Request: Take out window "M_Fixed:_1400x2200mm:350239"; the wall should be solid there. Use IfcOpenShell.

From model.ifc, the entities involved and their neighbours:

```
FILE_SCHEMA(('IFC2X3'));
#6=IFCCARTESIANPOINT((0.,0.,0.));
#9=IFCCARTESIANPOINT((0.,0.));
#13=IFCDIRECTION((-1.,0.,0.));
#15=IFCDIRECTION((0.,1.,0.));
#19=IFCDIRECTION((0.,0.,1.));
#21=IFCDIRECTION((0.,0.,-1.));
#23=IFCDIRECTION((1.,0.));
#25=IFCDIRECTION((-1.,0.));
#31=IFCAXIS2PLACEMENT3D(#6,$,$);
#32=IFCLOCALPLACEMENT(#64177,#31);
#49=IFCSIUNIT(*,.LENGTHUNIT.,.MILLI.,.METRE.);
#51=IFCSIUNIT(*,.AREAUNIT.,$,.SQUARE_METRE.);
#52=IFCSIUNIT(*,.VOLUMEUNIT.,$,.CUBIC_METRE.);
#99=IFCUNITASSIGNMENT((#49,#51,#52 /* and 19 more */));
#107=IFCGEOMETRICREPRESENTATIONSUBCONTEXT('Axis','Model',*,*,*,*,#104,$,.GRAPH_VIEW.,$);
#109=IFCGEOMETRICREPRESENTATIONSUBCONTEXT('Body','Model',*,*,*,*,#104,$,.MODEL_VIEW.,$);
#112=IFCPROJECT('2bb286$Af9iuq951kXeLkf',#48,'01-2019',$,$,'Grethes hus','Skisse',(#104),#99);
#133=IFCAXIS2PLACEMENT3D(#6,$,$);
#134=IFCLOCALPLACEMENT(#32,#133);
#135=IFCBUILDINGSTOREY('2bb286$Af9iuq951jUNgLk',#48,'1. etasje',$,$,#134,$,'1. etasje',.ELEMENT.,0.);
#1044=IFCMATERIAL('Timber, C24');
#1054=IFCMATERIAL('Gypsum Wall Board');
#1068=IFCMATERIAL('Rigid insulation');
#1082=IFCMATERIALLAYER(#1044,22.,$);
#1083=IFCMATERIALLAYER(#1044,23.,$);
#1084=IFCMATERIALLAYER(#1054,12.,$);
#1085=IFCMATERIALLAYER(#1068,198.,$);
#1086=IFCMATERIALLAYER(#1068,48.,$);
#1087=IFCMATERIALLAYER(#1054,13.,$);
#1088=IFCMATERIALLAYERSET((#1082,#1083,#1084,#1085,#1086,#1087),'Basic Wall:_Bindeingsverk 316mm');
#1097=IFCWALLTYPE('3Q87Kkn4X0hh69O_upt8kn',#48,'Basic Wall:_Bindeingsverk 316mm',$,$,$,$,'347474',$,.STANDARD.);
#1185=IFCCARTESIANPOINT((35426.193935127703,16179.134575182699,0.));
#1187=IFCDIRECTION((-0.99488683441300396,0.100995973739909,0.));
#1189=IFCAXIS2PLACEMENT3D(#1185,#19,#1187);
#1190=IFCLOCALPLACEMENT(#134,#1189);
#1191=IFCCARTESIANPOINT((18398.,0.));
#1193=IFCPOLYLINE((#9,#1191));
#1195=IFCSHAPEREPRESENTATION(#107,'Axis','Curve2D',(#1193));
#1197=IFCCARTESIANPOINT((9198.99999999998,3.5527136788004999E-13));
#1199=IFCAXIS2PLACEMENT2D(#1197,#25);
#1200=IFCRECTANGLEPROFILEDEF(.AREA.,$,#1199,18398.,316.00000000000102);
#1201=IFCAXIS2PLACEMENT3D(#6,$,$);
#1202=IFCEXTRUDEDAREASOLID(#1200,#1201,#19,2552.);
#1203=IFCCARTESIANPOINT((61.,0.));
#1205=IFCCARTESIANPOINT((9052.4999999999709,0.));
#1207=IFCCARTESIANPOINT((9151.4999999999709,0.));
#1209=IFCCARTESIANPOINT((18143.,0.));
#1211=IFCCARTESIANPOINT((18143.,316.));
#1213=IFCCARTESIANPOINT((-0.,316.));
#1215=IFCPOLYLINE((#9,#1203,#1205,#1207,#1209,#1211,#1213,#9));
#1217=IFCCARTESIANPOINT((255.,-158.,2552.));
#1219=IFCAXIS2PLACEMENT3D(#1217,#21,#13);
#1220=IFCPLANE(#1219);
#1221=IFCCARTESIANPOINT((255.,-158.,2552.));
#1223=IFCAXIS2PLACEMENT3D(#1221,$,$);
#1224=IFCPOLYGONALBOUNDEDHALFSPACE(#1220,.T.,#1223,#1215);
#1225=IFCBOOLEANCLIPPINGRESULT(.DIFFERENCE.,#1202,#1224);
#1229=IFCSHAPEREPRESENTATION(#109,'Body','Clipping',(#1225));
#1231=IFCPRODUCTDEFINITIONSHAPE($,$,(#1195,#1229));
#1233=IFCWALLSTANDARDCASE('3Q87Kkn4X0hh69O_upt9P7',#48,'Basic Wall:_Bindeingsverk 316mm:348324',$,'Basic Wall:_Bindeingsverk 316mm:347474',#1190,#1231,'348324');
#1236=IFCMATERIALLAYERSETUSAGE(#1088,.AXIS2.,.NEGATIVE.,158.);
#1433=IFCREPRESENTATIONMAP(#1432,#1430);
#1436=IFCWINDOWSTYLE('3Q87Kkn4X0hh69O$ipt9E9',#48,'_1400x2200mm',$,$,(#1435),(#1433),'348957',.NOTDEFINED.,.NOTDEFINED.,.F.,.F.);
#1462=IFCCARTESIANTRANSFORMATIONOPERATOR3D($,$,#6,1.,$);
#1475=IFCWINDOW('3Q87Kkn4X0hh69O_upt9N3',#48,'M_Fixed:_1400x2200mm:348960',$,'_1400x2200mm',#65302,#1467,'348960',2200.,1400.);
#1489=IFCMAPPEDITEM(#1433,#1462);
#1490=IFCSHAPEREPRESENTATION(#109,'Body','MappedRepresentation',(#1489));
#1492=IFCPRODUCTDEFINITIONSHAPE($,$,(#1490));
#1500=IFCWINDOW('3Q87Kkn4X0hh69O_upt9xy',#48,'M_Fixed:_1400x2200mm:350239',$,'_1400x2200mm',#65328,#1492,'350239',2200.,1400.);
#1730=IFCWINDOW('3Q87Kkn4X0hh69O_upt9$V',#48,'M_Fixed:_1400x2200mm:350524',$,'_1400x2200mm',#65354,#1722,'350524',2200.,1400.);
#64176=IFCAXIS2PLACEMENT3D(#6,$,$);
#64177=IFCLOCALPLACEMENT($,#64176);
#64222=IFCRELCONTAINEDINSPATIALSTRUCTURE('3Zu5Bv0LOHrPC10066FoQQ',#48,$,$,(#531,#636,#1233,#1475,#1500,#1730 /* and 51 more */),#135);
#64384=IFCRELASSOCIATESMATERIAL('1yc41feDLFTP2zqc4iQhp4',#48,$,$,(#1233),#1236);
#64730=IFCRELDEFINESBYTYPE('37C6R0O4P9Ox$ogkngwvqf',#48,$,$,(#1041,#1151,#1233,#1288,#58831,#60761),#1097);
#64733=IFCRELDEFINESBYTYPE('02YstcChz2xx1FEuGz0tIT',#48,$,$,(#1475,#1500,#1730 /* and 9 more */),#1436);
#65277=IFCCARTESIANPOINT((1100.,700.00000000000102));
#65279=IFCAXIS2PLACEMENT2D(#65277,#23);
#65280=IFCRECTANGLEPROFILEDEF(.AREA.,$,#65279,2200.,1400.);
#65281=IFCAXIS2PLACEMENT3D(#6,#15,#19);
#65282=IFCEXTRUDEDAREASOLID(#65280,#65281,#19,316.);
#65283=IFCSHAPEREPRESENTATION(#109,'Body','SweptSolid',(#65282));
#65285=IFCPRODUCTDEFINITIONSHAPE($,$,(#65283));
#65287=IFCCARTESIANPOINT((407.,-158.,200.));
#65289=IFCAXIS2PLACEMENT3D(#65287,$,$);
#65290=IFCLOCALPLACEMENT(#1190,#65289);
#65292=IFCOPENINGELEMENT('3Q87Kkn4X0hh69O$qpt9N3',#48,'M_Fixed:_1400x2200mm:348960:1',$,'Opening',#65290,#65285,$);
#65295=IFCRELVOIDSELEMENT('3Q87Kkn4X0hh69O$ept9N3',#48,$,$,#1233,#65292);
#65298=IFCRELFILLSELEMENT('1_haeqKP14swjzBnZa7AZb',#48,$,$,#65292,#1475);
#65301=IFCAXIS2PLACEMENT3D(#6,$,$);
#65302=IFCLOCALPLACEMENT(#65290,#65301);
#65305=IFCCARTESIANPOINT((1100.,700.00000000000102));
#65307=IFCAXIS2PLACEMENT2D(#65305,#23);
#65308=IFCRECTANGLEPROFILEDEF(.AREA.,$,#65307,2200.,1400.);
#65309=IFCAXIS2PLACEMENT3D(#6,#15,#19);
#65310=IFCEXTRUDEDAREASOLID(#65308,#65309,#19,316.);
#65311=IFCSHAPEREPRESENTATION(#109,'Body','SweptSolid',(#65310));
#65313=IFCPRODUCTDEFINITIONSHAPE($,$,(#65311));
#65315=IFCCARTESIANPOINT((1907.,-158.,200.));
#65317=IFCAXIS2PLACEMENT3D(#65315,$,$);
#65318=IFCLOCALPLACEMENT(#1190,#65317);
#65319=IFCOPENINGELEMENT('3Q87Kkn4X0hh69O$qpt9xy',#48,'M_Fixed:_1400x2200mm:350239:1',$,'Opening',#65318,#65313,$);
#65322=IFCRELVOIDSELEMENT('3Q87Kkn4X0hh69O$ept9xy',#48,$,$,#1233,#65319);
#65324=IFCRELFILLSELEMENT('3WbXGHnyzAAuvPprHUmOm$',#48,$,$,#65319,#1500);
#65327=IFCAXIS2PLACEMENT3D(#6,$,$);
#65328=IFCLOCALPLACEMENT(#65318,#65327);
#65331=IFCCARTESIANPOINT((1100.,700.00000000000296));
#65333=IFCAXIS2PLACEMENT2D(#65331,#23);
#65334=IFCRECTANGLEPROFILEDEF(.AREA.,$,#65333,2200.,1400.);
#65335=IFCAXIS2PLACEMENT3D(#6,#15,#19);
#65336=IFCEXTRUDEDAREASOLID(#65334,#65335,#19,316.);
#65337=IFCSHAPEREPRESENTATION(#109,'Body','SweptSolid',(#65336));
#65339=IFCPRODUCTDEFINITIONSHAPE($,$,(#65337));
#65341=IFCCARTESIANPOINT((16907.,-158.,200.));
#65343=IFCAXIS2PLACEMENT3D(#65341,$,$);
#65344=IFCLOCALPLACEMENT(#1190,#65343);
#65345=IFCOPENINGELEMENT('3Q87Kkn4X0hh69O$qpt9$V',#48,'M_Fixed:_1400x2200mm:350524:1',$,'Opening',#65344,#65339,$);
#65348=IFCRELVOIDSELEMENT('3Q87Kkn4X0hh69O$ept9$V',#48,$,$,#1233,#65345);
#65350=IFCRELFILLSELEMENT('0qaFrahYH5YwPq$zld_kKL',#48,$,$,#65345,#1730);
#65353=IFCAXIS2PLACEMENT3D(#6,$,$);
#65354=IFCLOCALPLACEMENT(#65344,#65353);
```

```python
import ifcopenshell
import ifcopenshell.api.feature
import ifcopenshell.api.root
import ifcopenshell.geom
import ifcopenshell.util.shape

model = ifcopenshell.open("model.ifc")
settings = ifcopenshell.geom.settings()


def volume(element):
    """Net volume in cubic metres, openings subtracted."""
    shape = ifcopenshell.geom.create_shape(settings, element)
    return ifcopenshell.util.shape.get_volume(shape.geometry)


window = model.by_guid("3Q87Kkn4X0hh69O_upt9xy")
opening = window.FillsVoids[0].RelatingOpeningElement
wall = opening.VoidsElements[0].RelatingBuildingElement
before = volume(wall)

ifcopenshell.api.root.remove_product(model, product=window)
ifcopenshell.api.feature.remove_feature(model, feature=opening)

after = volume(wall)

print(f"wall volume {before:.3f} -> {after:.3f} m3")

model.write("model_edited.ifc")
```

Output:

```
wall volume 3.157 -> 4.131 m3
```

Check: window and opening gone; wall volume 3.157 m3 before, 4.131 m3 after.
